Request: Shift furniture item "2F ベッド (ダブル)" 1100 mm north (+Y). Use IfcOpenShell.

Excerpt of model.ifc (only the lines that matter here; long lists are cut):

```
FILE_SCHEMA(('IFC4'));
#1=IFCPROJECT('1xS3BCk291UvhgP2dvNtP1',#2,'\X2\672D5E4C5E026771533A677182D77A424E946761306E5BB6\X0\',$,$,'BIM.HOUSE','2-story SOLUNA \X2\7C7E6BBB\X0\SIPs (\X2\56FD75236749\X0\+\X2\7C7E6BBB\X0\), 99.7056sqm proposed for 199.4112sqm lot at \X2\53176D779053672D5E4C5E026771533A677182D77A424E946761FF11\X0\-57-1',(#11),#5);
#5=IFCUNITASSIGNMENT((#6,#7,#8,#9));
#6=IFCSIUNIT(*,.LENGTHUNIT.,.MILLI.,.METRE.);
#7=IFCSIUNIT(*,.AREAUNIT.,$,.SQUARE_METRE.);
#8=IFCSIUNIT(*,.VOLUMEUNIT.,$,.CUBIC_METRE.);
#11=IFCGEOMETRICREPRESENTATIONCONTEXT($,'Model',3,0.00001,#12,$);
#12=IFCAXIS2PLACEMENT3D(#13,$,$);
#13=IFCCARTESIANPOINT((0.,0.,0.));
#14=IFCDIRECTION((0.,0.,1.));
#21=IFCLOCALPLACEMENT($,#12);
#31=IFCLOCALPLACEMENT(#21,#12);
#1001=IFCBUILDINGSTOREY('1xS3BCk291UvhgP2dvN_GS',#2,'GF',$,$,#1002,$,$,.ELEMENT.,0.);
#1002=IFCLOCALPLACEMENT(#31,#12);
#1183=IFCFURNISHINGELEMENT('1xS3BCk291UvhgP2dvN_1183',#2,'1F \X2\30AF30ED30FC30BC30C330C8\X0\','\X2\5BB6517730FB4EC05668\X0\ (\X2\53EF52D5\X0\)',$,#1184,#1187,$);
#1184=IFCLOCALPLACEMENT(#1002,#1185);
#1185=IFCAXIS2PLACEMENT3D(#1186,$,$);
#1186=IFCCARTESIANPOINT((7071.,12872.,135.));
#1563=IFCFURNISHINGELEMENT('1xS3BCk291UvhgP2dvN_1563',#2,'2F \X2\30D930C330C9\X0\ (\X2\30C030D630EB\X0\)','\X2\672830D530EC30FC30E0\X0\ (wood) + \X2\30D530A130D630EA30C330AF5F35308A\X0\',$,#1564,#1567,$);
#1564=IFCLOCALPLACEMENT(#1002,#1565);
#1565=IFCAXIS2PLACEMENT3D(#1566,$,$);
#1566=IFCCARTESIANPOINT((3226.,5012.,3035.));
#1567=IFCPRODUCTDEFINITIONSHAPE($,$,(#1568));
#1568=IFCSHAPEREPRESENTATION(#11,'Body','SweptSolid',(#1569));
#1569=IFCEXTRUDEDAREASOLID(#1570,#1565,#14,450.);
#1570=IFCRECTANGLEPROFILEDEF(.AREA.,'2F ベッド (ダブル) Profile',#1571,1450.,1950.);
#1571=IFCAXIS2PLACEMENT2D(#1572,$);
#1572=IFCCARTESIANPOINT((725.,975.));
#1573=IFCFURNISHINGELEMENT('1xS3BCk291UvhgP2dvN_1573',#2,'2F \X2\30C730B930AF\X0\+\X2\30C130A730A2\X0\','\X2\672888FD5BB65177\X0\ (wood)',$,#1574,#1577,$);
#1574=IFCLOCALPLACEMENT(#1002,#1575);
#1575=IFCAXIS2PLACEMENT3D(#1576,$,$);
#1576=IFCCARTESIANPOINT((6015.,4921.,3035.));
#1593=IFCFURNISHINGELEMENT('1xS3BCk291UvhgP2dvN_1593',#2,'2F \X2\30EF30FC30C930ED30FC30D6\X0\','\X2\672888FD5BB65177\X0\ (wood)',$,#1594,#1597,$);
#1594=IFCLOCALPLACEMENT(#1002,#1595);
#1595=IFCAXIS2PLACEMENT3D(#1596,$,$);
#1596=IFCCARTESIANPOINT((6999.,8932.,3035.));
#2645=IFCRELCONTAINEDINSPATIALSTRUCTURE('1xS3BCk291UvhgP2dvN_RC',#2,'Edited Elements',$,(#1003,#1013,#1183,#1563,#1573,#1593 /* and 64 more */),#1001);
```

```python
import ifcopenshell
import ifcopenshell.api.geometry
import ifcopenshell.util.placement

model = ifcopenshell.open("model.ifc")

item = model.by_guid("1xS3BCk291UvhgP2dvN_1563")
matrix = ifcopenshell.util.placement.get_local_placement(item.ObjectPlacement)
matrix[1, 3] += 1100.0
ifcopenshell.api.geometry.edit_object_placement(model, product=item, matrix=matrix, is_si=False)

print(ifcopenshell.util.placement.get_local_placement(item.ObjectPlacement).round(3) + 0.0)

model.write("model_updated.ifc")
```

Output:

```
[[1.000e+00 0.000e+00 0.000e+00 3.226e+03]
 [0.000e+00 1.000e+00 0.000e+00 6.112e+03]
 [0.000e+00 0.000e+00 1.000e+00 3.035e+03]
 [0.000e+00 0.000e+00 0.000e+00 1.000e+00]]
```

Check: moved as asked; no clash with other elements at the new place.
